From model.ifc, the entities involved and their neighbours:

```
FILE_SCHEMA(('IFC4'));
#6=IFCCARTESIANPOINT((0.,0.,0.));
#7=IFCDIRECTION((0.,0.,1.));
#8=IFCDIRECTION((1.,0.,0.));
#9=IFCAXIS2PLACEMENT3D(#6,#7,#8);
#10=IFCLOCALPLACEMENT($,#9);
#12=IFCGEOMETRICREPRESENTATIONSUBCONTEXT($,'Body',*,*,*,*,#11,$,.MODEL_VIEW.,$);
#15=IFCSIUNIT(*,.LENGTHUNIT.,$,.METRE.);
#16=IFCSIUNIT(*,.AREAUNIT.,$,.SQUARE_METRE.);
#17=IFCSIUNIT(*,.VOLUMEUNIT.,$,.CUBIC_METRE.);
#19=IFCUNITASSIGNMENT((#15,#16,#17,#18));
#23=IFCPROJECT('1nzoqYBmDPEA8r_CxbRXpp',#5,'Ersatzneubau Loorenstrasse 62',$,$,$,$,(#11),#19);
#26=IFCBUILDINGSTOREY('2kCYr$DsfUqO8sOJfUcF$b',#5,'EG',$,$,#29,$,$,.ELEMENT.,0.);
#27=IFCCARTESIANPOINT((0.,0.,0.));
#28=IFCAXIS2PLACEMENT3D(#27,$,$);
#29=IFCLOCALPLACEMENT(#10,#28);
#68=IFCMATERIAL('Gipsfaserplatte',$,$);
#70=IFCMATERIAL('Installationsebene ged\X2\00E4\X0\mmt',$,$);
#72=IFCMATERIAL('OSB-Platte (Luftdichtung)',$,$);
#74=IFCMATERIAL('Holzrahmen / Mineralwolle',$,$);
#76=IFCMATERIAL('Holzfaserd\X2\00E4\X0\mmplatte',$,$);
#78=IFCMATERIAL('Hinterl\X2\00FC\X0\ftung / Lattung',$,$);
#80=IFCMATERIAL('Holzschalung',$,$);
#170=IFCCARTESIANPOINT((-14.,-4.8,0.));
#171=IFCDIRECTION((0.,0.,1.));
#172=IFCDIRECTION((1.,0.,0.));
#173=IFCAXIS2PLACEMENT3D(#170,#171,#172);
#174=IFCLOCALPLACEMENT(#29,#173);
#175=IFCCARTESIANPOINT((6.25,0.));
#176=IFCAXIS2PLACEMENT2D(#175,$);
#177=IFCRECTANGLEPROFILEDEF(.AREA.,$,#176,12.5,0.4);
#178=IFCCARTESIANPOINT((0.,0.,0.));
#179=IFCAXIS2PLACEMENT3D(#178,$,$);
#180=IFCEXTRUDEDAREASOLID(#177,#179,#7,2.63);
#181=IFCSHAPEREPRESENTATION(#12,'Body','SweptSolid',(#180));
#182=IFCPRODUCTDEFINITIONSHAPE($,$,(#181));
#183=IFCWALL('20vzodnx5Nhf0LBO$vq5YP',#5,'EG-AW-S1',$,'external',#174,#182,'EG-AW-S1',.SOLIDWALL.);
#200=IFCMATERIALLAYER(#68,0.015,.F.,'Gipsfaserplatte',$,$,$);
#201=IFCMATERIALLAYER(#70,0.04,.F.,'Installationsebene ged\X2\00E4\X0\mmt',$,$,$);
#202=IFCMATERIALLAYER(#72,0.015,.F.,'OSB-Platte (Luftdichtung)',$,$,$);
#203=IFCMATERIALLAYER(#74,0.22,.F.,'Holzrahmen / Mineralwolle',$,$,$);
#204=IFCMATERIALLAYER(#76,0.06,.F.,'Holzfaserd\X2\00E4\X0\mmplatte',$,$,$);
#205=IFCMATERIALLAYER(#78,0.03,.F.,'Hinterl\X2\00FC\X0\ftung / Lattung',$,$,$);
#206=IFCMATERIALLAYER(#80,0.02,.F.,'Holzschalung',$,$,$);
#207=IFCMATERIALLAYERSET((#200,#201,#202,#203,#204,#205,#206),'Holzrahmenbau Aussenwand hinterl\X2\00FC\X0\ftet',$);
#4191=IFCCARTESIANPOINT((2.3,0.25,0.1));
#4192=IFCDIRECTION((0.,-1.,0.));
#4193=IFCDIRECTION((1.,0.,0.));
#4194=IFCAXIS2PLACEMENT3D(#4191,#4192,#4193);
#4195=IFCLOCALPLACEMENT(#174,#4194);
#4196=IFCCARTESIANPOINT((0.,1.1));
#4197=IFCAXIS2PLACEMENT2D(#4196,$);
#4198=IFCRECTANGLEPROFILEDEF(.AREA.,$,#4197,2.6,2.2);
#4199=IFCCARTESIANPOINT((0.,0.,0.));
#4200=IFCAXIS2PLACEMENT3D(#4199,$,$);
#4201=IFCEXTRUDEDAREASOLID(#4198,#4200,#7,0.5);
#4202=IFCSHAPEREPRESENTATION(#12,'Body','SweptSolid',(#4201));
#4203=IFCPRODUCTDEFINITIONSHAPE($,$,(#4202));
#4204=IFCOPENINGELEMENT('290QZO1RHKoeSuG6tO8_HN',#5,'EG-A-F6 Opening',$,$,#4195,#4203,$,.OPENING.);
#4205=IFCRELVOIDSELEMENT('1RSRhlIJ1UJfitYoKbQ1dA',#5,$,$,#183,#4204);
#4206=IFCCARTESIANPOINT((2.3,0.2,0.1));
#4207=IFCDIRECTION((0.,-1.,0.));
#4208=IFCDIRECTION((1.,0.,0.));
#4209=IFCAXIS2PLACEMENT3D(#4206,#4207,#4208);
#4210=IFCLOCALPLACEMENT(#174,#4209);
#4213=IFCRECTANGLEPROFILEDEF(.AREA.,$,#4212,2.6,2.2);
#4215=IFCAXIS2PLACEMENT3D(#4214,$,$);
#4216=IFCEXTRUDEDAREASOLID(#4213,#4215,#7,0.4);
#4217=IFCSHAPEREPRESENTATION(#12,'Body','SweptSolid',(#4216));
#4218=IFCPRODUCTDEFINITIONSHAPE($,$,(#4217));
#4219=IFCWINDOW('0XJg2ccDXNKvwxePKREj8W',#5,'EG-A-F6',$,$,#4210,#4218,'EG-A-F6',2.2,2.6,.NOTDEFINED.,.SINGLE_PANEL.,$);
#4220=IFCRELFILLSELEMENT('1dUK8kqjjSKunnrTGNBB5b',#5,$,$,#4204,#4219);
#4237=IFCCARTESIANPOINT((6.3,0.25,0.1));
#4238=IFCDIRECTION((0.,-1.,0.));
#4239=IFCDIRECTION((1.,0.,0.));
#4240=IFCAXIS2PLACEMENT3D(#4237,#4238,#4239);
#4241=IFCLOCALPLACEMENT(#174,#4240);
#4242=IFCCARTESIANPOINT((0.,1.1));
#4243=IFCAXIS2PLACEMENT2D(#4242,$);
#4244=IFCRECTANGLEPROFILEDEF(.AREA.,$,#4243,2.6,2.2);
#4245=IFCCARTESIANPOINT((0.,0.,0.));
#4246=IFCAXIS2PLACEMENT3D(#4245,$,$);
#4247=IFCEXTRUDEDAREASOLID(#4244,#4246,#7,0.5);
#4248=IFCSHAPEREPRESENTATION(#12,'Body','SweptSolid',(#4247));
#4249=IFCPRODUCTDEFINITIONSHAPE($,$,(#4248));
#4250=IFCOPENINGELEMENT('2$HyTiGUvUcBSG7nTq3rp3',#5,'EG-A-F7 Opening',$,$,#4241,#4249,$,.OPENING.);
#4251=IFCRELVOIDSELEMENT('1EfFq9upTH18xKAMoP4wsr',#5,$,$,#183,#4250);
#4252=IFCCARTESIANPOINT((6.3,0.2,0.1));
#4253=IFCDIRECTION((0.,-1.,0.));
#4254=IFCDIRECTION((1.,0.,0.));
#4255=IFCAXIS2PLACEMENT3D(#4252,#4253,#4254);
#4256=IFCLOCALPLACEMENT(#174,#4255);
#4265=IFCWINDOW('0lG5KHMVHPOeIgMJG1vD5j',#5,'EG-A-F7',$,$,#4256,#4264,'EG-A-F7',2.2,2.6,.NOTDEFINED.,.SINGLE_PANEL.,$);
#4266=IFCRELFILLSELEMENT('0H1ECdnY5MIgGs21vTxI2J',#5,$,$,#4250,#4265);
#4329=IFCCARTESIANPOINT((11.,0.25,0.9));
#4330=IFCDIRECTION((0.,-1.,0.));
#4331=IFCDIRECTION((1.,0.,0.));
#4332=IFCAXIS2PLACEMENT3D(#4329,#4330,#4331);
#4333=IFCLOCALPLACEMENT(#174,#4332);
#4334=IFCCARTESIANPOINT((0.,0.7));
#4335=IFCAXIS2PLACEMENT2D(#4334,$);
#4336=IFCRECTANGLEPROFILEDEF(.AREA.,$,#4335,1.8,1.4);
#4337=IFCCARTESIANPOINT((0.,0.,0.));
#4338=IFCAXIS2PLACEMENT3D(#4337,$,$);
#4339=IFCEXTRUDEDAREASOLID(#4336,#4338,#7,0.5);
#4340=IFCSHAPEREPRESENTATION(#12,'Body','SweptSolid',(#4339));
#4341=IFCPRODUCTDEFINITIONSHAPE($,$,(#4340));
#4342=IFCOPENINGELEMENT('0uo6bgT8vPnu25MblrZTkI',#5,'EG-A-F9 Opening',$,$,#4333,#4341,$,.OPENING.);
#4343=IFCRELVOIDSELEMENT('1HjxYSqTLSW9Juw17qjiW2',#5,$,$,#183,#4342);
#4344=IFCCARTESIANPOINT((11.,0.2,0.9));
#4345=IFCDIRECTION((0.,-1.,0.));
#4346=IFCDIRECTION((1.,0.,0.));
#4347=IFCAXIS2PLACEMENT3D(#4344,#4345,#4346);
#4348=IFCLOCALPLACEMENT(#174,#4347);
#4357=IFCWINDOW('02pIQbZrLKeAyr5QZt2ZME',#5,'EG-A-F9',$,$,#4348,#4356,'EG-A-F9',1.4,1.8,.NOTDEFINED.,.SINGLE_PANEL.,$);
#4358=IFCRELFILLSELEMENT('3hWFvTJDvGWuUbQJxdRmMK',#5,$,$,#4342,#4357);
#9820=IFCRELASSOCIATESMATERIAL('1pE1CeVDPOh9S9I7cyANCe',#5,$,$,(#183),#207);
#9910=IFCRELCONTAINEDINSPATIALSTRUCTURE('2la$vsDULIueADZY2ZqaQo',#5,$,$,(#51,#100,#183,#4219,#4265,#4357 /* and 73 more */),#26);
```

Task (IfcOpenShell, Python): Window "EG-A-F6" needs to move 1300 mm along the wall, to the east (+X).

```python
import ifcopenshell
import ifcopenshell.api.geometry
import ifcopenshell.util.placement
import ifcopenshell.util.unit

model = ifcopenshell.open("model.ifc")
unit_scale = ifcopenshell.util.unit.calculate_unit_scale(model)

window = model.by_guid("0XJg2ccDXNKvwxePKREj8W")
opening = window.FillsVoids[0].RelatingOpeningElement
wall = opening.VoidsElements[0].RelatingBuildingElement

wall_matrix = ifcopenshell.util.placement.get_local_placement(wall.ObjectPlacement)
shift = wall_matrix[:3, 0] * 1.3 / unit_scale
before = ifcopenshell.util.placement.get_local_placement(window.ObjectPlacement)[:3, 3].copy()

# The window is not placed relative to its opening, so move both.
for product in (opening, window):
    matrix = ifcopenshell.util.placement.get_local_placement(product.ObjectPlacement)
    matrix[:3, 3] += shift
    ifcopenshell.api.geometry.edit_object_placement(model, product=product, matrix=matrix, is_si=False)

after = ifcopenshell.util.placement.get_local_placement(window.ObjectPlacement)[:3, 3]
print("window moved by", (after - before).round(3) + 0.0)

model.write("model-out.ifc")
```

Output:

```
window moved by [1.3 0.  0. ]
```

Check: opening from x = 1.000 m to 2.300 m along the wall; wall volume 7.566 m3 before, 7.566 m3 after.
